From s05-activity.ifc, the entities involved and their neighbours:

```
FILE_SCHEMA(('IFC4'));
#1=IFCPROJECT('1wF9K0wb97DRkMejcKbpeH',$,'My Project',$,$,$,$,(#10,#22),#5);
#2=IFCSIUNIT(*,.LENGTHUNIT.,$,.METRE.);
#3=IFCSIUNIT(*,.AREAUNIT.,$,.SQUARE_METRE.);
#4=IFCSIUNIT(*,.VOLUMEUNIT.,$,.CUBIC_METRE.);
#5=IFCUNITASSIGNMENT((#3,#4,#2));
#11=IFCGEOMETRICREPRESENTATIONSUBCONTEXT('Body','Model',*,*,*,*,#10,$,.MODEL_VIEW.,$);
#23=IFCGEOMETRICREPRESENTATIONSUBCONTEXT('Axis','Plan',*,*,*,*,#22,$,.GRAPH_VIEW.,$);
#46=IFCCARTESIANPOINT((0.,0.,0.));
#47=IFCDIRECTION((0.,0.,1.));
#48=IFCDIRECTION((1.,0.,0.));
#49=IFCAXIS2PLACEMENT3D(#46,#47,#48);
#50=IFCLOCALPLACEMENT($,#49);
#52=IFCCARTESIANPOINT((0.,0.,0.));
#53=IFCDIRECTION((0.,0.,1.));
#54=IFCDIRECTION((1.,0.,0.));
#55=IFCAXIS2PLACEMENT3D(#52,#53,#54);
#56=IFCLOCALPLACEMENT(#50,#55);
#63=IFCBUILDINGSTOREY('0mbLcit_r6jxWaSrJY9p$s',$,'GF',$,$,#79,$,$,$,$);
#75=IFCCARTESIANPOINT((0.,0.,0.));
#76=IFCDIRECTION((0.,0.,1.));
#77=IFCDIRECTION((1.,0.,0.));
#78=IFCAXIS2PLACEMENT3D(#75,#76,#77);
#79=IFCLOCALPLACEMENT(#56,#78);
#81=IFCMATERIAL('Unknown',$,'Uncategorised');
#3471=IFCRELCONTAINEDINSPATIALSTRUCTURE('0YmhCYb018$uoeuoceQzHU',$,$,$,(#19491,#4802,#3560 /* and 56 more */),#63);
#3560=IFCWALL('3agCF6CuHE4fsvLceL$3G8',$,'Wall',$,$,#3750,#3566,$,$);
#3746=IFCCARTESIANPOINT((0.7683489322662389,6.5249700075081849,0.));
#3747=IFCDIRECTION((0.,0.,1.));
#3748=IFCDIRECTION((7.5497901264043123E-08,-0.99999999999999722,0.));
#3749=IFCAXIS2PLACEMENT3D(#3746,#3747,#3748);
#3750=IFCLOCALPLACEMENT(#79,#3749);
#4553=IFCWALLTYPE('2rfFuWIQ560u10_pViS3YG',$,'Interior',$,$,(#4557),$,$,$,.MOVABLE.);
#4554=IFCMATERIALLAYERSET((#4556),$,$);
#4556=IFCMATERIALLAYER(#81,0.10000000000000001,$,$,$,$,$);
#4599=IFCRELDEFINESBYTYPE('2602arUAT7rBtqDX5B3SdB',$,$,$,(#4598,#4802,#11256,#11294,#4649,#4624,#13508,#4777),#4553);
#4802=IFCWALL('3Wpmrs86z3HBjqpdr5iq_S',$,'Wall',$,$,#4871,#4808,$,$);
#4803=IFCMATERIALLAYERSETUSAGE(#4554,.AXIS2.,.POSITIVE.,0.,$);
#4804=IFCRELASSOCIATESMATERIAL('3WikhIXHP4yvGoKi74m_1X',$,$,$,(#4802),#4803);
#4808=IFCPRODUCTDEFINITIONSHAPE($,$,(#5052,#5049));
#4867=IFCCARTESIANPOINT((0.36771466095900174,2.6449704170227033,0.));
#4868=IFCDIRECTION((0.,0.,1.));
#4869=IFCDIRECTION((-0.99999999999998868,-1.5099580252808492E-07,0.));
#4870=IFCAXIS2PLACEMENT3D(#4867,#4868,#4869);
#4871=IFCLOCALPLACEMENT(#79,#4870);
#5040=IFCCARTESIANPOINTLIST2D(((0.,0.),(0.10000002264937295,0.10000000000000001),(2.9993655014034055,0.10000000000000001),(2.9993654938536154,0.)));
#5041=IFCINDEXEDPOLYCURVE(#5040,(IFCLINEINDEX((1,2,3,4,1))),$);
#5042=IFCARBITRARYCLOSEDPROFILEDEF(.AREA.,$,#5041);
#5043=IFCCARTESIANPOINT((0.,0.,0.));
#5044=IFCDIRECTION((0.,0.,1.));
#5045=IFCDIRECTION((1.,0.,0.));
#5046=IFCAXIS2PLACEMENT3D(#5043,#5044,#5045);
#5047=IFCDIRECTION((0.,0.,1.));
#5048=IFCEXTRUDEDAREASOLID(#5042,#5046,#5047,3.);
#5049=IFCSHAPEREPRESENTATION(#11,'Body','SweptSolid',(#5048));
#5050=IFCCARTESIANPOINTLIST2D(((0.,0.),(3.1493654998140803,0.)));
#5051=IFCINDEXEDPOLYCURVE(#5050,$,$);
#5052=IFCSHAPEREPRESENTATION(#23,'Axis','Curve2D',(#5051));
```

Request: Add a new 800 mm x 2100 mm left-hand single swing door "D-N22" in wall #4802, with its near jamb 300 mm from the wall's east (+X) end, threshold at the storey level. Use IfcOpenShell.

```python
import numpy as np
import ifcopenshell
import ifcopenshell.api.feature
import ifcopenshell.api.geometry
import ifcopenshell.api.root
import ifcopenshell.api.spatial
import ifcopenshell.geom
import ifcopenshell.util.element
import ifcopenshell.util.placement
import ifcopenshell.util.representation
import ifcopenshell.util.shape
import ifcopenshell.util.unit

model = ifcopenshell.open("s05-activity.ifc")
unit_scale = ifcopenshell.util.unit.calculate_unit_scale(model)
settings = ifcopenshell.geom.settings()


def volume(element):
    """Net volume in cubic metres, openings subtracted."""
    shape = ifcopenshell.geom.create_shape(settings, element)
    return ifcopenshell.util.shape.get_volume(shape.geometry)


wall = model.by_id(4802)
storey = ifcopenshell.util.element.get_container(wall, ifc_class="IfcBuildingStorey")
context = ifcopenshell.util.representation.get_context(model, "Model", "Body", "MODEL_VIEW")
before = volume(wall)

width, height, from_end, sill = 0.8, 2.1, 0.3, 0.0  # metres

# The wall runs along its own X axis, and the end named is its -X end.
wall_shape = ifcopenshell.geom.create_shape(settings, wall)
x, y, z = ifcopenshell.util.shape.get_vertices(wall_shape.geometry).T
start = x.min() + from_end
face, thickness = float(y.min()), float(y.max() - y.min())
wall_matrix = ifcopenshell.util.placement.get_local_placement(wall.ObjectPlacement)
level = ifcopenshell.util.placement.get_local_placement(storey.ObjectPlacement)[2, 3]


def in_wall(x, y):
    """Placement at x, y metres in the wall's axes, at sill height."""
    matrix = wall_matrix.copy()
    matrix[:, 3] = wall_matrix @ np.array([x / unit_scale, y / unit_scale, 0.0, 1.0])
    matrix[2, 3] = level + sill / unit_scale
    return matrix


# Opening: a box that overshoots both wall faces by 50 mm.
opening = ifcopenshell.api.root.create_entity(model, ifc_class="IfcOpeningElement", predefined_type="OPENING")
box = ifcopenshell.api.geometry.add_wall_representation(
    model, context=context, length=width, height=height, thickness=thickness + 0.1
)
ifcopenshell.api.geometry.assign_representation(model, product=opening, representation=box)
ifcopenshell.api.geometry.edit_object_placement(model, product=opening, matrix=in_wall(start, face - 0.05), is_si=False)
ifcopenshell.api.feature.add_feature(model, feature=opening, element=wall)

door = ifcopenshell.api.root.create_entity(model, ifc_class="IfcDoor", name="D-N22", predefined_type="DOOR")
door.OverallWidth, door.OverallHeight = width / unit_scale, height / unit_scale
door.OperationType = "SINGLE_SWING_LEFT"
body = ifcopenshell.api.geometry.add_door_representation(
    model,
    context=context,
    overall_width=door.OverallWidth,
    overall_height=door.OverallHeight,
    operation_type="SINGLE_SWING_LEFT",
    lining_properties={"LiningDepth": thickness / unit_scale, "ThresholdDepth": thickness / unit_scale},
)
ifcopenshell.api.geometry.assign_representation(model, product=door, representation=body)
ifcopenshell.api.spatial.assign_container(model, products=[door], relating_structure=storey)
ifcopenshell.api.feature.add_filling(model, opening=opening, element=door)

# The lining spans the wall, so the door starts at the wall face.
ifcopenshell.api.geometry.edit_object_placement(model, product=door, matrix=in_wall(start, face), is_si=False)

after = volume(wall)

print(f"wall volume {before:.3f} -> {after:.3f} m3")

model.write("s05-activity_rev.ifc")
```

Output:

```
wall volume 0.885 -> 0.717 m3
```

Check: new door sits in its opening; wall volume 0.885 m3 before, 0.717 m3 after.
